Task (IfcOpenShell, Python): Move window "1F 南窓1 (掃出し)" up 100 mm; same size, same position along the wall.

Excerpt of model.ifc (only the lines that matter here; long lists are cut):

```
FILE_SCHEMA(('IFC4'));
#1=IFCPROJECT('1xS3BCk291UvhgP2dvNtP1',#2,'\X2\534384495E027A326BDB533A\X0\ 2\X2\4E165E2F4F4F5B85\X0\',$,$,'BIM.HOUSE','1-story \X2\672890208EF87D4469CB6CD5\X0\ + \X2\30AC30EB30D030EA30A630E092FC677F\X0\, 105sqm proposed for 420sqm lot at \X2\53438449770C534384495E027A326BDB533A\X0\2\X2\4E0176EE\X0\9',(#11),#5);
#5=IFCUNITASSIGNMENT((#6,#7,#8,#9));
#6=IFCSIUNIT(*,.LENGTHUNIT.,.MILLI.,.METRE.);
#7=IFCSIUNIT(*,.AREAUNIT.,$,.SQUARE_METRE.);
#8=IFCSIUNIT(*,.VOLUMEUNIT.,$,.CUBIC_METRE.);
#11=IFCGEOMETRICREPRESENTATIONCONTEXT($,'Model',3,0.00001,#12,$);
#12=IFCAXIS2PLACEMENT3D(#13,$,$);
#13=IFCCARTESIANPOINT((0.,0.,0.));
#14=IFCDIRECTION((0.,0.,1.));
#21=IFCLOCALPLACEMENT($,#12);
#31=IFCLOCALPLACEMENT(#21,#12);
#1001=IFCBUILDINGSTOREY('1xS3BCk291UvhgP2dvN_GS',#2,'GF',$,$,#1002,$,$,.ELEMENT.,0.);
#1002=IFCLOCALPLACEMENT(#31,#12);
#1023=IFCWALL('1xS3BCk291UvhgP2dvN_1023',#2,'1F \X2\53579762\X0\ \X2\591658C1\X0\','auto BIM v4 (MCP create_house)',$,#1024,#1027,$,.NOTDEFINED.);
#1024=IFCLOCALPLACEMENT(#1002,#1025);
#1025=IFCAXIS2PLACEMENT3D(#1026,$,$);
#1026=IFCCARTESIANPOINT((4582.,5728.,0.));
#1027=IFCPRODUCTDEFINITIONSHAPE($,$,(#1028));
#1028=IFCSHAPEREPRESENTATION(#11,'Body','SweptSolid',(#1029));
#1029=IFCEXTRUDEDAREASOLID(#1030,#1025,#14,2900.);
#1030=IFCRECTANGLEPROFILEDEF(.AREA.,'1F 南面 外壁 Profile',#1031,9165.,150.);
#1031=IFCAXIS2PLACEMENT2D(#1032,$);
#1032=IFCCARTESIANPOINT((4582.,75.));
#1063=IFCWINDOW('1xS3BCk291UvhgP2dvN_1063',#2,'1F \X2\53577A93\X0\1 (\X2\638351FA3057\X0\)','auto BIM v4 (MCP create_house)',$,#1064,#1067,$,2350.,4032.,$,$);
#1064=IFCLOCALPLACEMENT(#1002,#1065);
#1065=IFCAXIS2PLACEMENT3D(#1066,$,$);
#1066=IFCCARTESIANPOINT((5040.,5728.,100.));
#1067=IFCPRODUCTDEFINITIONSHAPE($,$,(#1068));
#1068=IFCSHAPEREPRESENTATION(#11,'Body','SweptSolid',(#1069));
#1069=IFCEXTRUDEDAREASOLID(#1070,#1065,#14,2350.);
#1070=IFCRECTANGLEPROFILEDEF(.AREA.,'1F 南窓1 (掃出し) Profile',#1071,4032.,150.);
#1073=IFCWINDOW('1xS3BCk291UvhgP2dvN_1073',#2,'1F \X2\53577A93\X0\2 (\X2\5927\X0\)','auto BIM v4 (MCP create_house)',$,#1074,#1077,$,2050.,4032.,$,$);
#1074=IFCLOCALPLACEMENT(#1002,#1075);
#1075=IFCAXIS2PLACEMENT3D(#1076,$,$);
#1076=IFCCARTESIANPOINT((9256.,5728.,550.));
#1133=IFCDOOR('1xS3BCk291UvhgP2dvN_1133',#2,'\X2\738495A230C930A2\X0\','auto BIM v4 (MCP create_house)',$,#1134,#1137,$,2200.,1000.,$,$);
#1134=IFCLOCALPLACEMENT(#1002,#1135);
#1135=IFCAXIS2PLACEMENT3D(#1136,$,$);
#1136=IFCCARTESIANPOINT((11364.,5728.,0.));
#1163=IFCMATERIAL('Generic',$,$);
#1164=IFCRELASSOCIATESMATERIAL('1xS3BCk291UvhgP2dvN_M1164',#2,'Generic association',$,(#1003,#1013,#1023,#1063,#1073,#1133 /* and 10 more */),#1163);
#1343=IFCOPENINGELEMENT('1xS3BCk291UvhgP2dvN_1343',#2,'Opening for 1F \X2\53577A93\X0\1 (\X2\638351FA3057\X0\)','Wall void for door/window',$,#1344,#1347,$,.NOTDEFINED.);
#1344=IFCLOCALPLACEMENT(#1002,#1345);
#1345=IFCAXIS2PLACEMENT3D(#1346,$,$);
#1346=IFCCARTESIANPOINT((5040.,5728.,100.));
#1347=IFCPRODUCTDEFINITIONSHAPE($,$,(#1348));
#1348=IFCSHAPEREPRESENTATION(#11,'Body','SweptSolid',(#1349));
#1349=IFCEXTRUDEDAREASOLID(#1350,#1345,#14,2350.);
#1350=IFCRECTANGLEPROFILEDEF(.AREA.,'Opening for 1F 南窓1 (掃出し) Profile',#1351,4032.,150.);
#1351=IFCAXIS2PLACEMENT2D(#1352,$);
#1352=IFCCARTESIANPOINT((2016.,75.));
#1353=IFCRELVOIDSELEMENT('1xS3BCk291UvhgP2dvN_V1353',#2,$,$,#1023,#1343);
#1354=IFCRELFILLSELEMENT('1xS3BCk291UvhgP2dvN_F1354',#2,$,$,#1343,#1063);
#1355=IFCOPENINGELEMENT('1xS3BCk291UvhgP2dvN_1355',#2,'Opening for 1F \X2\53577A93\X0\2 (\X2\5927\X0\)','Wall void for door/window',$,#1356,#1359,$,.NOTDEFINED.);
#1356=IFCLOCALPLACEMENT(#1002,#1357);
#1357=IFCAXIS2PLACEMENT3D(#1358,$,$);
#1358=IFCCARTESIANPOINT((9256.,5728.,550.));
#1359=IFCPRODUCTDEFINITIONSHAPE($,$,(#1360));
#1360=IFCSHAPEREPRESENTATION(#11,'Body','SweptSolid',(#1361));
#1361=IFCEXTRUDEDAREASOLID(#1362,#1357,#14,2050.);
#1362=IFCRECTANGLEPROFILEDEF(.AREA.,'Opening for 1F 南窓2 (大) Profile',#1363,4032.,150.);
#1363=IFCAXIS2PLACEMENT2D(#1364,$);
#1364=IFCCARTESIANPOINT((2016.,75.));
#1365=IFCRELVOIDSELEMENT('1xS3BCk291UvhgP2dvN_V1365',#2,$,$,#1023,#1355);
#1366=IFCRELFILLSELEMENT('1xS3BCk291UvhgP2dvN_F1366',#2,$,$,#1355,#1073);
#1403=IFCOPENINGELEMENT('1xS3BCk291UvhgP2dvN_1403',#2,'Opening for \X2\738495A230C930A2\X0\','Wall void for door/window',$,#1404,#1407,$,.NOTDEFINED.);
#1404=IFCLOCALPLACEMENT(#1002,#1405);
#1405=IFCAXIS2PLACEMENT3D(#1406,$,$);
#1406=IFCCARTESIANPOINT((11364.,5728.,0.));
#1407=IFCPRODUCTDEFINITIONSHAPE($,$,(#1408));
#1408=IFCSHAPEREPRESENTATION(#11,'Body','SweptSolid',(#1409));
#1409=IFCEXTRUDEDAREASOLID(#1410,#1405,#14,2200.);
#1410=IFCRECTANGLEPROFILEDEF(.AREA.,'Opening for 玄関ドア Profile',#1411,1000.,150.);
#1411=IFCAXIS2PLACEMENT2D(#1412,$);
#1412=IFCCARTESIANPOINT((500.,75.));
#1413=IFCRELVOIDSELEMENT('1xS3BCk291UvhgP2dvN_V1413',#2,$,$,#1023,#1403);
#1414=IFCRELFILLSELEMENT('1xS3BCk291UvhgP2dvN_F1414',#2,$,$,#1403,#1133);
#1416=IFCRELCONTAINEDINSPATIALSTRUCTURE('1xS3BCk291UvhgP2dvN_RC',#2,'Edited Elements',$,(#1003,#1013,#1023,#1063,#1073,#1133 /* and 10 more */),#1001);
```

```python
import numpy as np
import ifcopenshell
import ifcopenshell.api.geometry
import ifcopenshell.util.placement
import ifcopenshell.util.unit

model = ifcopenshell.open("model.ifc")
unit_scale = ifcopenshell.util.unit.calculate_unit_scale(model)

window = model.by_guid("1xS3BCk291UvhgP2dvN_1063")
opening = window.FillsVoids[0].RelatingOpeningElement
dz = 0.1 / unit_scale

shift = np.array([0.0, 0.0, dz])
# The window is not placed relative to its opening, so move both.
for product in (opening, window):
    matrix = ifcopenshell.util.placement.get_local_placement(product.ObjectPlacement)
    matrix[:3, 3] += shift
    ifcopenshell.api.geometry.edit_object_placement(model, product=product, matrix=matrix, is_si=False)

print(f"moved by {dz * unit_scale:+.3f} m")

model.write("model-out.ifc")
```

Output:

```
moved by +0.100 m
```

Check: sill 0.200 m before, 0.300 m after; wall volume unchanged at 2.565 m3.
